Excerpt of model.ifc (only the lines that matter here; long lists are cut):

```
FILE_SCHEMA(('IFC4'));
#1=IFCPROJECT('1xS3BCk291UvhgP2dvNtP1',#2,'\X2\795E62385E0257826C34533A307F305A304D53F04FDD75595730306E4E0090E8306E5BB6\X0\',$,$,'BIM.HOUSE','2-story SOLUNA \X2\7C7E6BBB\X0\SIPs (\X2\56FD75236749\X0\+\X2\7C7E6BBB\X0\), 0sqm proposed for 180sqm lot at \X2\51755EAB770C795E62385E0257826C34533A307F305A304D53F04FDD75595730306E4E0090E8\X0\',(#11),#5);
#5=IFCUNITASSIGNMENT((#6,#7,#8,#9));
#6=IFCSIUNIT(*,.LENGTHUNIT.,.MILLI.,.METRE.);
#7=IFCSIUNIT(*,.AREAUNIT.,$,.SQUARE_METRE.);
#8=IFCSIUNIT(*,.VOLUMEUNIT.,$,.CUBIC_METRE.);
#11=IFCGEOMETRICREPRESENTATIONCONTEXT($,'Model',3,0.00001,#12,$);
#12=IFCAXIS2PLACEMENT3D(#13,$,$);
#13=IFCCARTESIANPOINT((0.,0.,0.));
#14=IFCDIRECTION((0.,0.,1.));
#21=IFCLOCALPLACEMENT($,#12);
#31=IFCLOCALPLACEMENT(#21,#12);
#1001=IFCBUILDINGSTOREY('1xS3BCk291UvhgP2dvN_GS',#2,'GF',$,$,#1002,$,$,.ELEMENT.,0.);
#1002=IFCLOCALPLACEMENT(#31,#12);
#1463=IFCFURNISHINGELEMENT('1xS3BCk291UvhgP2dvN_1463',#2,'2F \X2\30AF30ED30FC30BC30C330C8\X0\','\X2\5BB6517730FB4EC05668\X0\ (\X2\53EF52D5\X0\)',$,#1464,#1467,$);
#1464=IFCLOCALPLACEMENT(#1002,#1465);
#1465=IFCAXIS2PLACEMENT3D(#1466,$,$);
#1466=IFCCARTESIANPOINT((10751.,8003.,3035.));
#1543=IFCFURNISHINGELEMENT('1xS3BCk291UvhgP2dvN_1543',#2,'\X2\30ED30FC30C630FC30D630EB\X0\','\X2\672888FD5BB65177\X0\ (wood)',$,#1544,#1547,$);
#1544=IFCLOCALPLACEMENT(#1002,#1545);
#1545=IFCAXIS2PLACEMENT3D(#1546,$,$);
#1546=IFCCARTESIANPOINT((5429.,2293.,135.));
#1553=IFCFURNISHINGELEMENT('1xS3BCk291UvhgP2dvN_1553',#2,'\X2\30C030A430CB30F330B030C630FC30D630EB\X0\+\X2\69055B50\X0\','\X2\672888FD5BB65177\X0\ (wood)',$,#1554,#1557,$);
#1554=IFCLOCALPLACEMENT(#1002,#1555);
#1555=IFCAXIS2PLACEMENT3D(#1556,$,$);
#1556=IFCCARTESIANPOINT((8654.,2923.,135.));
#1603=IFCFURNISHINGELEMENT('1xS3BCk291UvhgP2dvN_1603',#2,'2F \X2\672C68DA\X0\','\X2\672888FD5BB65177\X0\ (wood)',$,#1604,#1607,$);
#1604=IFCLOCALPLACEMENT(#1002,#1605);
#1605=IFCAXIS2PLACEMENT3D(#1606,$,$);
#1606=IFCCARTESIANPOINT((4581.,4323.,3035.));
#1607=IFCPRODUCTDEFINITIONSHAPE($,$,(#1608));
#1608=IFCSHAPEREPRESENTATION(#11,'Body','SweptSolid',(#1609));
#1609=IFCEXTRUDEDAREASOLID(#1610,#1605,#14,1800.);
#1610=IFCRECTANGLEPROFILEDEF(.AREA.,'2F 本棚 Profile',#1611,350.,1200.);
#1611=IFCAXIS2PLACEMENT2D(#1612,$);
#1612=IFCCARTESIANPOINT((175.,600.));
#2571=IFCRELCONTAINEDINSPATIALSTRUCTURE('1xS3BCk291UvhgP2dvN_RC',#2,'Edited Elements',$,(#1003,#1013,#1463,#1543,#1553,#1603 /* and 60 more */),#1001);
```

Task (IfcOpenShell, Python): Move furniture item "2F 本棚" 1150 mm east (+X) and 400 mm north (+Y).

```python
import ifcopenshell
import ifcopenshell.api.geometry
import ifcopenshell.util.placement

model = ifcopenshell.open("model.ifc")

item = model.by_guid("1xS3BCk291UvhgP2dvN_1603")
matrix = ifcopenshell.util.placement.get_local_placement(item.ObjectPlacement)
matrix[0, 3] += 1150.0
matrix[1, 3] += 400.0
ifcopenshell.api.geometry.edit_object_placement(model, product=item, matrix=matrix, is_si=False)

print(ifcopenshell.util.placement.get_local_placement(item.ObjectPlacement).round(3) + 0.0)

model.write("model_rev.ifc")
```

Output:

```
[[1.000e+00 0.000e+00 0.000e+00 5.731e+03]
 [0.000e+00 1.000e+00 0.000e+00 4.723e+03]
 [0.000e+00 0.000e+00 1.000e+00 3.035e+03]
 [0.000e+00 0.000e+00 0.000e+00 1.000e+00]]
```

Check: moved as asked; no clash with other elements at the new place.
